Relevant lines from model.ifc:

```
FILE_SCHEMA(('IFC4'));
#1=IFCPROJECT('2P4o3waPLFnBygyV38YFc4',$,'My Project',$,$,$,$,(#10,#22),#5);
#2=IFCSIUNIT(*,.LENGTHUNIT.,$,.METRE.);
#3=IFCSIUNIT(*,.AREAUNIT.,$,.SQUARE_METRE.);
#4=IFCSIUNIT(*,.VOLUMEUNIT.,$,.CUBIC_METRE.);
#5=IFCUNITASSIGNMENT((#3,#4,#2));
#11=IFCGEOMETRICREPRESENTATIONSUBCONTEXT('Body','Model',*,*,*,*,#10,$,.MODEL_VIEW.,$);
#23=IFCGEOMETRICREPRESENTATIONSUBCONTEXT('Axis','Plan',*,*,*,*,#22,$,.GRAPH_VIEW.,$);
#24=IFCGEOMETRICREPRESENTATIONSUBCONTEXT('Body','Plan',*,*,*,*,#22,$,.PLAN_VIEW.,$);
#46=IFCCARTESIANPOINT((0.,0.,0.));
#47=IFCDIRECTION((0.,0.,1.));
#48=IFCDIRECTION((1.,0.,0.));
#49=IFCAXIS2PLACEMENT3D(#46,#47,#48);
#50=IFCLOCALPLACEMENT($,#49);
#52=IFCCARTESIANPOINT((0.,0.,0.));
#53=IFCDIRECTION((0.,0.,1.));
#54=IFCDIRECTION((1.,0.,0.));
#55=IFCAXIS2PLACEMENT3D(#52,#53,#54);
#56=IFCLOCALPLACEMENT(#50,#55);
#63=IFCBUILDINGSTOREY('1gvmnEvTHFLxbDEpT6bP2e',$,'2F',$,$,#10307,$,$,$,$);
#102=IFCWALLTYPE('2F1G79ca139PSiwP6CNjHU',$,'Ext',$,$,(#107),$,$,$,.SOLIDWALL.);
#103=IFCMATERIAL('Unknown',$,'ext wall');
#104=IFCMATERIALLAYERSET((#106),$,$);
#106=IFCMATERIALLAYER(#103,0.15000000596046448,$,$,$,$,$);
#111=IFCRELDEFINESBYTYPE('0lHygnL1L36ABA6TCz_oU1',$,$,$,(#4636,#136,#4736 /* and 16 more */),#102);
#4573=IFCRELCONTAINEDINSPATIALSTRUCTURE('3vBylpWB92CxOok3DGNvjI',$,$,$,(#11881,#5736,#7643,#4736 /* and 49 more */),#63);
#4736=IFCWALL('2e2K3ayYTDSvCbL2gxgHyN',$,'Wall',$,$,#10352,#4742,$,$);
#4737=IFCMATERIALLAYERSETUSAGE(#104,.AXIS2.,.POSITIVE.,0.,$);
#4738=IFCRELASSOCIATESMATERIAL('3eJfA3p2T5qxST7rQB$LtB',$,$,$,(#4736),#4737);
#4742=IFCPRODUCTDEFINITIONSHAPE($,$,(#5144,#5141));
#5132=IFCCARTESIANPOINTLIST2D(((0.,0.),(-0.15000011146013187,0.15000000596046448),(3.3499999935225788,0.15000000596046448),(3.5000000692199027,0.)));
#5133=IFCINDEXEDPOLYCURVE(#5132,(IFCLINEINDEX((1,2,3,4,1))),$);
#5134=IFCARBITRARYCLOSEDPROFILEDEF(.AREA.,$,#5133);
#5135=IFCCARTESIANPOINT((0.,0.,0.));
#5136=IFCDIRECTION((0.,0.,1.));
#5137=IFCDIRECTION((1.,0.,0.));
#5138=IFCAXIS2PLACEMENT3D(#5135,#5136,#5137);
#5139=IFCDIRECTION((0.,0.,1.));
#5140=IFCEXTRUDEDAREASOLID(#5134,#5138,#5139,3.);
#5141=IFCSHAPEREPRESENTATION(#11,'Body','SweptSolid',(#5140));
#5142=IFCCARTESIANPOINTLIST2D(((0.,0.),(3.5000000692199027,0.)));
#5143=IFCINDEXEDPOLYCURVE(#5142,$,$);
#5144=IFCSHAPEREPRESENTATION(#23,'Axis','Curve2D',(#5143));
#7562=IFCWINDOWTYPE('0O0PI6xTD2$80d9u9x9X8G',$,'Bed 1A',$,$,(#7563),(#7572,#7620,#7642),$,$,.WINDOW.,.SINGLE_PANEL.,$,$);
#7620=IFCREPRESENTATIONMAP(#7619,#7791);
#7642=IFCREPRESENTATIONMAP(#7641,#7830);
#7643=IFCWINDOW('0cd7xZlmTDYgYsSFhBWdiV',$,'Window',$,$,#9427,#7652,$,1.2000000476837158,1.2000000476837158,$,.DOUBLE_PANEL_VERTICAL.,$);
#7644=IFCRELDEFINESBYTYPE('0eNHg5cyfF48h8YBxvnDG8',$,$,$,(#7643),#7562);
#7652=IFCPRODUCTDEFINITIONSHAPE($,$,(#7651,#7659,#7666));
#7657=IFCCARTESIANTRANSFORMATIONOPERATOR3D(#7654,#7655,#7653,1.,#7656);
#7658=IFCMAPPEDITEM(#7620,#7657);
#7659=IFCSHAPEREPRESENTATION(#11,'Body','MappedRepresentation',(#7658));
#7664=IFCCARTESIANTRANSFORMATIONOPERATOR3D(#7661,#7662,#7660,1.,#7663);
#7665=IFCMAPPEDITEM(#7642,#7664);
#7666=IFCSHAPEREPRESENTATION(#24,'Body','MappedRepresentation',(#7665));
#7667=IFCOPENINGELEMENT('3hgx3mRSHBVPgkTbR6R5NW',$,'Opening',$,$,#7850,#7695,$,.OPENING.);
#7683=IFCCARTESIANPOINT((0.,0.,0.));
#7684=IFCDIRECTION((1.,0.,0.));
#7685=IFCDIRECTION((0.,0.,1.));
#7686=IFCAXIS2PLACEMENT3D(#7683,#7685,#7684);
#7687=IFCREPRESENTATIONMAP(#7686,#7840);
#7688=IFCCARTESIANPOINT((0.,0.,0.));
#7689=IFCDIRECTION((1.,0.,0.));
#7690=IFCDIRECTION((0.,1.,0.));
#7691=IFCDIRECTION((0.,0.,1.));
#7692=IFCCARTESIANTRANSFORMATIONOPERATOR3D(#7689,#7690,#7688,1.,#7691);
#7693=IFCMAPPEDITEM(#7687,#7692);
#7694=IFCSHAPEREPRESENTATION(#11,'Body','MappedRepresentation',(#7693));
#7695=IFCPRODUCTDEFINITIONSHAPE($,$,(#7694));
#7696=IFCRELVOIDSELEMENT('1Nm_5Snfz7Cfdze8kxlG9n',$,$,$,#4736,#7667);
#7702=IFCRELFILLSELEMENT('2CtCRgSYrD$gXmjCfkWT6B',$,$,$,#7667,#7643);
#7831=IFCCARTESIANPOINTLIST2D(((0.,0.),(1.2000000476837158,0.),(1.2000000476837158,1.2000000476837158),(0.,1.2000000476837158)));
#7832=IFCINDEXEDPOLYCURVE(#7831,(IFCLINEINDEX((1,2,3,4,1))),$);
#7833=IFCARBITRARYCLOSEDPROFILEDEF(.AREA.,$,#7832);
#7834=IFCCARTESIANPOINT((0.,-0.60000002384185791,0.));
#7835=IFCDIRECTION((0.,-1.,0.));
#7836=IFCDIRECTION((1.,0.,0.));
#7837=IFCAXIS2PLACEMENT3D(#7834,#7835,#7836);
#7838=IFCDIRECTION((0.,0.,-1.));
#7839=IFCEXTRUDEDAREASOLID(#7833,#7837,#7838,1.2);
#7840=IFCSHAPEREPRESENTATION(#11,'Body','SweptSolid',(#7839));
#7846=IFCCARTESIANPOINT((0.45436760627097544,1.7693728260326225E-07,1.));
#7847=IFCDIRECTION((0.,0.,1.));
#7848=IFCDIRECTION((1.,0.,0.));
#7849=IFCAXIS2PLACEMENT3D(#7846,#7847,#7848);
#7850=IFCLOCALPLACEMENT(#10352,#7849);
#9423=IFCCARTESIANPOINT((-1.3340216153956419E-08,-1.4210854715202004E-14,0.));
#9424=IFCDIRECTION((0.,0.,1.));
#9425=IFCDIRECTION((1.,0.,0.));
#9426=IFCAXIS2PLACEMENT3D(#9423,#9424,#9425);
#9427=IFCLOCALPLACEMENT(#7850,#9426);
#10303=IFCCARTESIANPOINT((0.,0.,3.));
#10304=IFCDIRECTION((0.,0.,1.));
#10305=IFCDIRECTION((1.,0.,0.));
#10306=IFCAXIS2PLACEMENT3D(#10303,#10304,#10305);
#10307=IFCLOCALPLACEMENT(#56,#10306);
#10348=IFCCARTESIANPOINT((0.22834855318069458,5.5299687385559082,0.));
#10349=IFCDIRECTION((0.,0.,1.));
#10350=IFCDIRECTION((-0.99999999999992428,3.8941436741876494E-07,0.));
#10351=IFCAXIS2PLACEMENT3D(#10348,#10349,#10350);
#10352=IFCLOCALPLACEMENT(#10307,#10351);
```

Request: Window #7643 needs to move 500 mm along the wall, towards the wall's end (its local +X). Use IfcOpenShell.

```python
import ifcopenshell
import ifcopenshell.api.geometry
import ifcopenshell.util.placement
import ifcopenshell.util.unit

model = ifcopenshell.open("model.ifc")
unit_scale = ifcopenshell.util.unit.calculate_unit_scale(model)

window = model.by_guid("0cd7xZlmTDYgYsSFhBWdiV")
opening = window.FillsVoids[0].RelatingOpeningElement
wall = opening.VoidsElements[0].RelatingBuildingElement

wall_matrix = ifcopenshell.util.placement.get_local_placement(wall.ObjectPlacement)
shift = wall_matrix[:3, 0] * 0.5 / unit_scale
before = ifcopenshell.util.placement.get_local_placement(window.ObjectPlacement)[:3, 3].copy()

# The window is placed relative to its opening, so it follows when the opening moves.
matrix = ifcopenshell.util.placement.get_local_placement(opening.ObjectPlacement)
matrix[:3, 3] += shift
ifcopenshell.api.geometry.edit_object_placement(
    model, product=opening, matrix=matrix, is_si=False, should_transform_children=True
)

after = ifcopenshell.util.placement.get_local_placement(window.ObjectPlacement)[:3, 3]
print("window moved by", (after - before).round(3) + 0.0)

model.write("model_v2.ifc")
```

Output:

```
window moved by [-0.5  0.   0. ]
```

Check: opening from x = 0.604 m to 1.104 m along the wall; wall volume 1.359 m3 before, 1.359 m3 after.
